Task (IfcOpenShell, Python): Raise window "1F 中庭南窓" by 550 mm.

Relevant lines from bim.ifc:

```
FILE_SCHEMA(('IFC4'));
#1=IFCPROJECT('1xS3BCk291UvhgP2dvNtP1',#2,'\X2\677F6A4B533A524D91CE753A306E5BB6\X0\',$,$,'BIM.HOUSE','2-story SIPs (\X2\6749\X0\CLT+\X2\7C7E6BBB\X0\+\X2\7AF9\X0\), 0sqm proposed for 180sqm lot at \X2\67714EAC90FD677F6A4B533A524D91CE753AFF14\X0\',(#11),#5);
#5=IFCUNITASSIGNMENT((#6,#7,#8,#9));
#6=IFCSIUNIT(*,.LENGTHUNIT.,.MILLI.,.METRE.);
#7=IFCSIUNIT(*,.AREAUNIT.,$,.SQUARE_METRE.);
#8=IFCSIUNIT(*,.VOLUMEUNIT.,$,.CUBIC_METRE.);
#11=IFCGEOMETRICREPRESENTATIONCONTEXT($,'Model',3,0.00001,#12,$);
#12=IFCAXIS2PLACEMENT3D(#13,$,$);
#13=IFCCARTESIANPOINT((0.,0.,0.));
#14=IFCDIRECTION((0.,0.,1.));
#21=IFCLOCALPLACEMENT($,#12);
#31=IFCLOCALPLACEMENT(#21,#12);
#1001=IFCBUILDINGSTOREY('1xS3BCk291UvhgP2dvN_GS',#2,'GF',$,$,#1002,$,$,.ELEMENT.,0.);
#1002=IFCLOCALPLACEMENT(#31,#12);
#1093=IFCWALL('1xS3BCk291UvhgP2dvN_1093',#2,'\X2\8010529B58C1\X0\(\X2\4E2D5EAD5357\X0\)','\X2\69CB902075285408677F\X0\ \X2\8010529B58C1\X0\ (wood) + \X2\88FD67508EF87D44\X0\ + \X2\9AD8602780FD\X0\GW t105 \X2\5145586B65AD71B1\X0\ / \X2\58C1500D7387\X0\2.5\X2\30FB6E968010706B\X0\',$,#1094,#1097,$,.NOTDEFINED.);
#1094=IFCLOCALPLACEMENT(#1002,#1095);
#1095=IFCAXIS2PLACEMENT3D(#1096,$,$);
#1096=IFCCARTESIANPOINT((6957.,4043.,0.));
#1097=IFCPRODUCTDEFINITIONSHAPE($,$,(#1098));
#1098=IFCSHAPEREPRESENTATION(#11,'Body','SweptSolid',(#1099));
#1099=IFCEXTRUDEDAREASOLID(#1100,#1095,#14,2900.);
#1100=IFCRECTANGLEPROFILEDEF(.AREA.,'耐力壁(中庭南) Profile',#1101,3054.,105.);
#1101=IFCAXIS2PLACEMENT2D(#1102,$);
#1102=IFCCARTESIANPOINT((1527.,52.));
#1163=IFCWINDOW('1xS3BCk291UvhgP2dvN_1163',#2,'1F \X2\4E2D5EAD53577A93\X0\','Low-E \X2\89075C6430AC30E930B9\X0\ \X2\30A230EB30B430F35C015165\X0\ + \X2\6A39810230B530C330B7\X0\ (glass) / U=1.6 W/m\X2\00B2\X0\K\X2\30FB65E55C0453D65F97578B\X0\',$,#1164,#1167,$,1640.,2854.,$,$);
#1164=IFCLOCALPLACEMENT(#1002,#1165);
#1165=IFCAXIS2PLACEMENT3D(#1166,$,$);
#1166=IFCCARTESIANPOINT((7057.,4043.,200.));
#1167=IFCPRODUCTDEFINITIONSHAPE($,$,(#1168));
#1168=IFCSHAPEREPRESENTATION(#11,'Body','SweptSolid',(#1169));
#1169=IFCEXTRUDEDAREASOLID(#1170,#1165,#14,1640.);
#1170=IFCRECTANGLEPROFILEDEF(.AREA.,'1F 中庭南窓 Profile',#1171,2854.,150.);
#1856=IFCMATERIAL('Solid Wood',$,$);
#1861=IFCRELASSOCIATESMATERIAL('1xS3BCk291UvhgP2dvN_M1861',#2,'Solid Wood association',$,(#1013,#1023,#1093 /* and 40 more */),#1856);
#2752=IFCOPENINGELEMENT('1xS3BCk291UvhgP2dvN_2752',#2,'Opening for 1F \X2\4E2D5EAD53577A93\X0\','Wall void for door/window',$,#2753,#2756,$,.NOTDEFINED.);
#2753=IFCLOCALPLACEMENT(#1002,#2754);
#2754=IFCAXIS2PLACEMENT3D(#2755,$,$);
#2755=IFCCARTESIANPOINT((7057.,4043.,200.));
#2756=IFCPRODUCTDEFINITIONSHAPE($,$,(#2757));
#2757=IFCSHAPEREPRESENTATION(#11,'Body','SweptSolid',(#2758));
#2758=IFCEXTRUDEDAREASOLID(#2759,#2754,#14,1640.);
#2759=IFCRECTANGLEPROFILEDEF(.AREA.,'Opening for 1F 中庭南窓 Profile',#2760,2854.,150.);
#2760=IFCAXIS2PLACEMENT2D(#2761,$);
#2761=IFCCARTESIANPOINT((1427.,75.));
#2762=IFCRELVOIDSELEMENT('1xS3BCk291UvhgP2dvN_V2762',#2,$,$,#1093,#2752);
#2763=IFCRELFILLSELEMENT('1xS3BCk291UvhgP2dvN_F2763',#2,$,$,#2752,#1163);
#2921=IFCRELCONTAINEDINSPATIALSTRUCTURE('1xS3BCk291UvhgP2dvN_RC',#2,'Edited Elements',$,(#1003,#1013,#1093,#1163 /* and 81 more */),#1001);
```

```python
import numpy as np
import ifcopenshell
import ifcopenshell.api.geometry
import ifcopenshell.util.placement
import ifcopenshell.util.unit

model = ifcopenshell.open("bim.ifc")
unit_scale = ifcopenshell.util.unit.calculate_unit_scale(model)

window = model.by_guid("1xS3BCk291UvhgP2dvN_1163")
opening = window.FillsVoids[0].RelatingOpeningElement
dz = 550.0

shift = np.array([0.0, 0.0, dz])
# The window is not placed relative to its opening, so move both.
for product in (opening, window):
    matrix = ifcopenshell.util.placement.get_local_placement(product.ObjectPlacement)
    matrix[:3, 3] += shift
    ifcopenshell.api.geometry.edit_object_placement(model, product=product, matrix=matrix, is_si=False)

print(f"moved by {dz * unit_scale:+.3f} m")

model.write("bim_rev.ifc")
```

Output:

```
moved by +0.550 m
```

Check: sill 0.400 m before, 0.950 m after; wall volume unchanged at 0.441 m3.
